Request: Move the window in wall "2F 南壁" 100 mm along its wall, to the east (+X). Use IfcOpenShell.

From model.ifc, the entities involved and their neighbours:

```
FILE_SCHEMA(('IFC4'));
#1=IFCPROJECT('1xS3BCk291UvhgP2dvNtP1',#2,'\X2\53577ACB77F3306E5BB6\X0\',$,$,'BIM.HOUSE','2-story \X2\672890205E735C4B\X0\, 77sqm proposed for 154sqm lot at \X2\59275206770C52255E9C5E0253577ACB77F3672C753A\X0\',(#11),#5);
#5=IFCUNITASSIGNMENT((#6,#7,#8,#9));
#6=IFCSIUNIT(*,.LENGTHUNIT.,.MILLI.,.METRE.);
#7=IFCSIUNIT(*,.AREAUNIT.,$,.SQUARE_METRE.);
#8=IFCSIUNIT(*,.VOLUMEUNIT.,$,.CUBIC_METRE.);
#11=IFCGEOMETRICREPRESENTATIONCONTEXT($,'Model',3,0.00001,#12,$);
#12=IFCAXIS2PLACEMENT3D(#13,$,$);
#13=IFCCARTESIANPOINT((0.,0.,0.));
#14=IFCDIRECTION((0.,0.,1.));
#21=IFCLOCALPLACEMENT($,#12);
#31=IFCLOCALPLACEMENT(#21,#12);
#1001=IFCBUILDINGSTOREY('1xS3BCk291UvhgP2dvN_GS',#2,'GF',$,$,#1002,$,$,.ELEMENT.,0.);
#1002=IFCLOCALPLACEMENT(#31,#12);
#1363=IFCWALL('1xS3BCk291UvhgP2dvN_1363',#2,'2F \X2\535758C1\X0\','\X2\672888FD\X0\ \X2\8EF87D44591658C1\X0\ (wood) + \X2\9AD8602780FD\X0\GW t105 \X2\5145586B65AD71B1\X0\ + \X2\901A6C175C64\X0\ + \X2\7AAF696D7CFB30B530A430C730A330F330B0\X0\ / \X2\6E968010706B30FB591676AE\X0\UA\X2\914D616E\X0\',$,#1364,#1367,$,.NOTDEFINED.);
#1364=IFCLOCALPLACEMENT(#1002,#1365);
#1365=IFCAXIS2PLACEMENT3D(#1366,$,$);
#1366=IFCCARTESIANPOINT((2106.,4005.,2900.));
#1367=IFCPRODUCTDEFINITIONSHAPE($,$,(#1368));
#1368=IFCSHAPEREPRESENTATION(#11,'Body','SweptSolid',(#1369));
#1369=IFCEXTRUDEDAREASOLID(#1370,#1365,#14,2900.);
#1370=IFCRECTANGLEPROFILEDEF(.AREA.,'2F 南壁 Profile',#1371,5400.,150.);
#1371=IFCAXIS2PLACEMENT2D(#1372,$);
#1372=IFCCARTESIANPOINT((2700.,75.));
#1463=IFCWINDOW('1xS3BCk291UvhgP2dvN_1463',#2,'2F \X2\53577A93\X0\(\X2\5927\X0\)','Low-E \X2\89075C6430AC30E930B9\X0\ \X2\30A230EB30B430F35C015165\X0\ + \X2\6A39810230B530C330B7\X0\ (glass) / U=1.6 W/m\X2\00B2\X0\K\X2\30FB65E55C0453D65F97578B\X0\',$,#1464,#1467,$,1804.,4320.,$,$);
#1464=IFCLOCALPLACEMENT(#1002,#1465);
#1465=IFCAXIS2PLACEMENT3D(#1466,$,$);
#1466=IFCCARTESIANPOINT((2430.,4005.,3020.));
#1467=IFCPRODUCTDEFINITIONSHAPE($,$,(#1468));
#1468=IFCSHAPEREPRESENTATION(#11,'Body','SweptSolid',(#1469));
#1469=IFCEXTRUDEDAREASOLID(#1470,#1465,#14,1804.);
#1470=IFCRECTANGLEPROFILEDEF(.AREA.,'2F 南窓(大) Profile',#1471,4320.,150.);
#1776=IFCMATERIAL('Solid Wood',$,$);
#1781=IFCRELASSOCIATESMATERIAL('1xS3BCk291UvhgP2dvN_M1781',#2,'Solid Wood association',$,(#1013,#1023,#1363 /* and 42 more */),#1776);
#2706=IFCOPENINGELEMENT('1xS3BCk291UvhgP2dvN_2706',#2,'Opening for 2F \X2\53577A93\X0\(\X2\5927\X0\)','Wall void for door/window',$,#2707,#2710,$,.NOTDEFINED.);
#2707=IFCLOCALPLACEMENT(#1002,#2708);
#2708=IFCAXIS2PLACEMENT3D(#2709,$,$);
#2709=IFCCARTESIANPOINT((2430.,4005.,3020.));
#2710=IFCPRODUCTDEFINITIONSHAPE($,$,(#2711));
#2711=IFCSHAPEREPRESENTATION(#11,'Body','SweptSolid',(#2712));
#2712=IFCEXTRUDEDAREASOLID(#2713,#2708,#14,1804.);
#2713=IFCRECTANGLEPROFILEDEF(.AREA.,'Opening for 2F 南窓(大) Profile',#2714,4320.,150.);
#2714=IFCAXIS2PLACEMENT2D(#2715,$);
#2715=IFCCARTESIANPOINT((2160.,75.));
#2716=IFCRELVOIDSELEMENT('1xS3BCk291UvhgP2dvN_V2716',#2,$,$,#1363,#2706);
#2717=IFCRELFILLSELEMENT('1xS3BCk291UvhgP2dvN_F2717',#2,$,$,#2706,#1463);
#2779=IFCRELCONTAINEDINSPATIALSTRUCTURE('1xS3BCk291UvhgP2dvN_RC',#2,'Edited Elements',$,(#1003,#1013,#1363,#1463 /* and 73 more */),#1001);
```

```python
import ifcopenshell
import ifcopenshell.api.geometry
import ifcopenshell.util.placement
import ifcopenshell.util.unit

model = ifcopenshell.open("model.ifc")
unit_scale = ifcopenshell.util.unit.calculate_unit_scale(model)

window = model.by_guid("1xS3BCk291UvhgP2dvN_1463")
opening = window.FillsVoids[0].RelatingOpeningElement
wall = opening.VoidsElements[0].RelatingBuildingElement

wall_matrix = ifcopenshell.util.placement.get_local_placement(wall.ObjectPlacement)
shift = wall_matrix[:3, 0] * 0.1 / unit_scale
before = ifcopenshell.util.placement.get_local_placement(window.ObjectPlacement)[:3, 3].copy()

# The window is not placed relative to its opening, so move both.
for product in (opening, window):
    matrix = ifcopenshell.util.placement.get_local_placement(product.ObjectPlacement)
    matrix[:3, 3] += shift
    ifcopenshell.api.geometry.edit_object_placement(model, product=product, matrix=matrix, is_si=False)

after = ifcopenshell.util.placement.get_local_placement(window.ObjectPlacement)[:3, 3]
print("window moved by", (after - before).round(3) + 0.0)

model.write("model-out.ifc")
```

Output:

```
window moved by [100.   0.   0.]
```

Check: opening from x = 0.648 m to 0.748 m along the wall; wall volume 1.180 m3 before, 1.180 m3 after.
